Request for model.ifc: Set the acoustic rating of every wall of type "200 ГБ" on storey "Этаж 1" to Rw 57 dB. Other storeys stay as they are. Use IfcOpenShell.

First a look at what the model holds.

```python
import ifcopenshell
import ifcopenshell.util.element

model = ifcopenshell.open("model.ifc")
print(model.schema)
storey = next(s for s in model.by_type("IfcBuildingStorey") if s.Name == "Этаж 1")
walls = [e for e in ifcopenshell.util.element.get_decomposition(storey) if e.is_a("IfcWall")]
seen = {}
for e in walls:
    element_type = ifcopenshell.util.element.get_type(e)
    key = (element_type.Name if element_type != e and element_type else None, ifcopenshell.util.element.get_pset(e, "Pset_WallCommon", "AcousticRating"))
    seen[key] = seen.get(key, 0) + 1
for (name, value), count in sorted(seen.items(), key=str):
    print(count, "x", name, "|", value)
```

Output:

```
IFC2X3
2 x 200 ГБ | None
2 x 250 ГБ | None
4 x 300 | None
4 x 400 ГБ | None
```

```python
import ifcopenshell
import ifcopenshell.api.pset
import ifcopenshell.util.element

model = ifcopenshell.open("model.ifc")

storey = next(s for s in model.by_type("IfcBuildingStorey") if s.Name == "Этаж 1")
walls = [e for e in ifcopenshell.util.element.get_decomposition(storey) if e.is_a("IfcWall")]

count = 0
for e in walls:
    element_type = ifcopenshell.util.element.get_type(e)
    if element_type in (None, e) or element_type.Name != "200 ГБ":
        continue
    # add_pset returns the element's existing set when there is one.
    pset = ifcopenshell.api.pset.add_pset(model, product=e, name="Pset_WallCommon")
    ifcopenshell.api.pset.edit_pset(model, pset=pset, properties={"AcousticRating": "Rw 57 dB"})
    count += 1

print(count, "walls updated")

model.write("model_updated.ifc")
```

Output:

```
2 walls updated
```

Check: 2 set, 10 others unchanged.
